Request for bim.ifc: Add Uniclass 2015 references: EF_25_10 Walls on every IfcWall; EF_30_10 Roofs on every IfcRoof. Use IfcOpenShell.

First a look at what the model holds.

```python
import ifcopenshell

model = ifcopenshell.open("bim.ifc")
print(model.schema)
print("classifications:", [c.Name for c in model.by_type("IfcClassification")])
for ifc_class in ("IfcDoor", "IfcRoof", "IfcStair", "IfcWall", "IfcWindow"):
    print(ifc_class, len(model.by_type(ifc_class)))
```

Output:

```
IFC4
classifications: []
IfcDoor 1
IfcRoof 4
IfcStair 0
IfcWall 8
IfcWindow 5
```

```python
import ifcopenshell
import ifcopenshell.api.classification

model = ifcopenshell.open("bim.ifc")

system = ifcopenshell.api.classification.add_classification(model, classification="Uniclass 2015")

codes = {
    "IfcWall": ("EF_25_10", "Walls"),
    "IfcRoof": ("EF_30_10", "Roofs"),
}
for ifc_class, (code, name) in codes.items():
    products = model.by_type(ifc_class)
    ifcopenshell.api.classification.add_reference(
        model, products=products, classification=system, identification=code, name=name
    )
    print(code, len(products))

model.write("bim_updated.ifc")
```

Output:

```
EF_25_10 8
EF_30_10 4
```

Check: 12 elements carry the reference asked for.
